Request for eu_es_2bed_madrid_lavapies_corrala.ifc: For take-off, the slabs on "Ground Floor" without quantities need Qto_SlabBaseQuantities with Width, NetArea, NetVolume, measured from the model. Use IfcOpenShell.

First a look at what the model holds.

```python
import ifcopenshell
import ifcopenshell.util.element
import ifcopenshell.util.unit

model = ifcopenshell.open("eu_es_2bed_madrid_lavapies_corrala.ifc")
print(model.schema)
for unit_type in ("LENGTHUNIT", "AREAUNIT", "VOLUMEUNIT"):
    print(unit_type, ifcopenshell.util.unit.calculate_unit_scale(model, unit_type))
storey = next(s for s in model.by_type("IfcBuildingStorey") if s.Name == "Ground Floor")
slabs = [e for e in ifcopenshell.util.element.get_decomposition(storey) if e.is_a("IfcSlab")]
for e in sorted(slabs, key=lambda e: e.id()):
    print(e.id(), e.is_a(), e.Name, list(ifcopenshell.util.element.get_psets(e, qtos_only=True)), sep=" | ")
```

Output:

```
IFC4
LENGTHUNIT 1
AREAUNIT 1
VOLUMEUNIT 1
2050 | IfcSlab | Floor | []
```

```python
import ifcopenshell
import ifcopenshell.api.pset
import ifcopenshell.geom
import ifcopenshell.util.element
import ifcopenshell.util.shape
import ifcopenshell.util.unit

model = ifcopenshell.open("eu_es_2bed_madrid_lavapies_corrala.ifc")
unit_scale = ifcopenshell.util.unit.calculate_unit_scale(model)
area_scale = ifcopenshell.util.unit.calculate_unit_scale(model, "AREAUNIT")
volume_scale = ifcopenshell.util.unit.calculate_unit_scale(model, "VOLUMEUNIT")
settings = ifcopenshell.geom.settings()

storey = next(s for s in model.by_type("IfcBuildingStorey") if s.Name == "Ground Floor")
slabs = [e for e in ifcopenshell.util.element.get_decomposition(storey) if e.is_a("IfcSlab")]

for e in sorted(slabs, key=lambda e: e.id()):
    if ifcopenshell.util.element.get_psets(e, qtos_only=True, should_inherit=False):
        continue
    # Geometry comes back in metres, in the element's own axes.
    shape = ifcopenshell.geom.create_shape(settings, e)
    values = {
        "Width": ifcopenshell.util.shape.get_z(shape.geometry) / unit_scale,
        "NetArea": ifcopenshell.util.shape.get_footprint_area(shape.geometry) / area_scale,
        "NetVolume": ifcopenshell.util.shape.get_volume(shape.geometry) / volume_scale,
    }
    qto = ifcopenshell.api.pset.add_qto(model, product=e, name="Qto_SlabBaseQuantities")
    ifcopenshell.api.pset.edit_qto(model, qto=qto, properties=values)
    print(e.id(), {k: round(v, 3) for k, v in values.items()})

model.write("eu_es_2bed_madrid_lavapies_corrala-out.ifc")
```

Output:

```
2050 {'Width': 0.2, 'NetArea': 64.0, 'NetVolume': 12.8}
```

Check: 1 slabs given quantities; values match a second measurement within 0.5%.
